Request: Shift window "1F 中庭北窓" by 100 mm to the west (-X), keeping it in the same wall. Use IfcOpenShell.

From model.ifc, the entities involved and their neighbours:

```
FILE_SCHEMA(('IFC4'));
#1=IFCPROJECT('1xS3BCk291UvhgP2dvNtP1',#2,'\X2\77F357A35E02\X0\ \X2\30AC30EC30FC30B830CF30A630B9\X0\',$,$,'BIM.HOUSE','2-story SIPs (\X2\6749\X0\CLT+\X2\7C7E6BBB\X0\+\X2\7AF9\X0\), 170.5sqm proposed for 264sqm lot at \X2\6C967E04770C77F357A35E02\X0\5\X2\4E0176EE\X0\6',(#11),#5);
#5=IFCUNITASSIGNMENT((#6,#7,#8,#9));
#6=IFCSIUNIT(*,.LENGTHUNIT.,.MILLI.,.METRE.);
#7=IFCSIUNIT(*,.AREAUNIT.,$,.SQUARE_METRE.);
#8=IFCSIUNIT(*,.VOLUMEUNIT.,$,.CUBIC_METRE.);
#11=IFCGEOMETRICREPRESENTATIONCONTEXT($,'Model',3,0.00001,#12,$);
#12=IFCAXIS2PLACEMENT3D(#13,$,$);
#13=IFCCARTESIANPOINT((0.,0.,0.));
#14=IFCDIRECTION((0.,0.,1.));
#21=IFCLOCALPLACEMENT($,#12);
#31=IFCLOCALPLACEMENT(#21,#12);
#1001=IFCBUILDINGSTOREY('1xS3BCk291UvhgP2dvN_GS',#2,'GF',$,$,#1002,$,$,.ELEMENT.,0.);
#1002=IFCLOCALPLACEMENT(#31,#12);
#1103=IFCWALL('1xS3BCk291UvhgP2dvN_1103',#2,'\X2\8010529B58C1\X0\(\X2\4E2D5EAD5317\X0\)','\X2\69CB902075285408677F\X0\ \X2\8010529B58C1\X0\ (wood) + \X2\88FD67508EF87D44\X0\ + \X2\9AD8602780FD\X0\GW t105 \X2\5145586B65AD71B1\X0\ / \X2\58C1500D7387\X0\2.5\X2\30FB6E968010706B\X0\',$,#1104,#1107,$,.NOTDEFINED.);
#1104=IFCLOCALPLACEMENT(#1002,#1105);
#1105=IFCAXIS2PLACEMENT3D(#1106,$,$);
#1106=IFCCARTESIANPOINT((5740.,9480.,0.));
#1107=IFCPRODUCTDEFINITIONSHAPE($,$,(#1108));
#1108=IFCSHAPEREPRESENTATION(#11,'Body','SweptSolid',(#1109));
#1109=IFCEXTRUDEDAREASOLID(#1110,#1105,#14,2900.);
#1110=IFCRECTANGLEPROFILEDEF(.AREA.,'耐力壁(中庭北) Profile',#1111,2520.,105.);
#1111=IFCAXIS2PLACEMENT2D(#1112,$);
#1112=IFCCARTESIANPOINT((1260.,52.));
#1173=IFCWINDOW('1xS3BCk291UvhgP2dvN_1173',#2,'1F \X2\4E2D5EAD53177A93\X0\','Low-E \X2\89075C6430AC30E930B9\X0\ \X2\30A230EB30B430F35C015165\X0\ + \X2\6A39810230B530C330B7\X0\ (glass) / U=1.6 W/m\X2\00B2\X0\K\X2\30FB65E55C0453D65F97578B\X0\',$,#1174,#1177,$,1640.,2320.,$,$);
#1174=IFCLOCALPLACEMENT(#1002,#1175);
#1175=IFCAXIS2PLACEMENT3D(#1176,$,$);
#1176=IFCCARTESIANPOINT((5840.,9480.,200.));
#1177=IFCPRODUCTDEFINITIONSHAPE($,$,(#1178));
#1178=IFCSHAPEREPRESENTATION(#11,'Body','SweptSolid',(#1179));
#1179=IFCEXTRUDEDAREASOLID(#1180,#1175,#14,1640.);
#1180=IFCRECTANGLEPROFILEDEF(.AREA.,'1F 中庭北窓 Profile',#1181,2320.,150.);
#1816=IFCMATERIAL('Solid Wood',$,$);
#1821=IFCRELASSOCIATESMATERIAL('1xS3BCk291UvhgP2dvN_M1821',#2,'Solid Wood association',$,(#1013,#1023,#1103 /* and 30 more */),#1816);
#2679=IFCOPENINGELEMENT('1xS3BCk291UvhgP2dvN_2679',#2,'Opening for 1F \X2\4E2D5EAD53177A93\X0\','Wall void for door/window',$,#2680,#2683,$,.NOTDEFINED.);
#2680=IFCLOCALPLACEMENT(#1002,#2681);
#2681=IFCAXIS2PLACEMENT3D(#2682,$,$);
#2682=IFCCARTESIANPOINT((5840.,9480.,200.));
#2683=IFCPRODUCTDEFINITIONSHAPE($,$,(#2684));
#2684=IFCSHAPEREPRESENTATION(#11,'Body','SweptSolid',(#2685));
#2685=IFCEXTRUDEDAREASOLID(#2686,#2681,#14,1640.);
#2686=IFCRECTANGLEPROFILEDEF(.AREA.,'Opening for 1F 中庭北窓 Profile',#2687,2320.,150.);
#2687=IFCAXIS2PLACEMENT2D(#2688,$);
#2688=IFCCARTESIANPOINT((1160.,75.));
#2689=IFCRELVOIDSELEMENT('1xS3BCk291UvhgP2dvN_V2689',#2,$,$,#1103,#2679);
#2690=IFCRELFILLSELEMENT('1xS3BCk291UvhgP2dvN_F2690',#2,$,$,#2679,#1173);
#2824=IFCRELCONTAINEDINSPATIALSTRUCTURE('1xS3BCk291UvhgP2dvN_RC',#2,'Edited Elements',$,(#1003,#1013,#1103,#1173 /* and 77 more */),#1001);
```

```python
import ifcopenshell
import ifcopenshell.api.geometry
import ifcopenshell.util.placement
import ifcopenshell.util.unit

model = ifcopenshell.open("model.ifc")
unit_scale = ifcopenshell.util.unit.calculate_unit_scale(model)

window = model.by_guid("1xS3BCk291UvhgP2dvN_1173")
opening = window.FillsVoids[0].RelatingOpeningElement
wall = opening.VoidsElements[0].RelatingBuildingElement

wall_matrix = ifcopenshell.util.placement.get_local_placement(wall.ObjectPlacement)
shift = wall_matrix[:3, 0] * -0.1 / unit_scale
before = ifcopenshell.util.placement.get_local_placement(window.ObjectPlacement)[:3, 3].copy()

# The window is not placed relative to its opening, so move both.
for product in (opening, window):
    matrix = ifcopenshell.util.placement.get_local_placement(product.ObjectPlacement)
    matrix[:3, 3] += shift
    ifcopenshell.api.geometry.edit_object_placement(model, product=product, matrix=matrix, is_si=False)

after = ifcopenshell.util.placement.get_local_placement(window.ObjectPlacement)[:3, 3]
print("window moved by", (after - before).round(3) + 0.0)

model.write("model_edited.ifc")
```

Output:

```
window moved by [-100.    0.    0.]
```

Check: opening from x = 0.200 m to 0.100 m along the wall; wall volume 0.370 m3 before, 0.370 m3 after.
